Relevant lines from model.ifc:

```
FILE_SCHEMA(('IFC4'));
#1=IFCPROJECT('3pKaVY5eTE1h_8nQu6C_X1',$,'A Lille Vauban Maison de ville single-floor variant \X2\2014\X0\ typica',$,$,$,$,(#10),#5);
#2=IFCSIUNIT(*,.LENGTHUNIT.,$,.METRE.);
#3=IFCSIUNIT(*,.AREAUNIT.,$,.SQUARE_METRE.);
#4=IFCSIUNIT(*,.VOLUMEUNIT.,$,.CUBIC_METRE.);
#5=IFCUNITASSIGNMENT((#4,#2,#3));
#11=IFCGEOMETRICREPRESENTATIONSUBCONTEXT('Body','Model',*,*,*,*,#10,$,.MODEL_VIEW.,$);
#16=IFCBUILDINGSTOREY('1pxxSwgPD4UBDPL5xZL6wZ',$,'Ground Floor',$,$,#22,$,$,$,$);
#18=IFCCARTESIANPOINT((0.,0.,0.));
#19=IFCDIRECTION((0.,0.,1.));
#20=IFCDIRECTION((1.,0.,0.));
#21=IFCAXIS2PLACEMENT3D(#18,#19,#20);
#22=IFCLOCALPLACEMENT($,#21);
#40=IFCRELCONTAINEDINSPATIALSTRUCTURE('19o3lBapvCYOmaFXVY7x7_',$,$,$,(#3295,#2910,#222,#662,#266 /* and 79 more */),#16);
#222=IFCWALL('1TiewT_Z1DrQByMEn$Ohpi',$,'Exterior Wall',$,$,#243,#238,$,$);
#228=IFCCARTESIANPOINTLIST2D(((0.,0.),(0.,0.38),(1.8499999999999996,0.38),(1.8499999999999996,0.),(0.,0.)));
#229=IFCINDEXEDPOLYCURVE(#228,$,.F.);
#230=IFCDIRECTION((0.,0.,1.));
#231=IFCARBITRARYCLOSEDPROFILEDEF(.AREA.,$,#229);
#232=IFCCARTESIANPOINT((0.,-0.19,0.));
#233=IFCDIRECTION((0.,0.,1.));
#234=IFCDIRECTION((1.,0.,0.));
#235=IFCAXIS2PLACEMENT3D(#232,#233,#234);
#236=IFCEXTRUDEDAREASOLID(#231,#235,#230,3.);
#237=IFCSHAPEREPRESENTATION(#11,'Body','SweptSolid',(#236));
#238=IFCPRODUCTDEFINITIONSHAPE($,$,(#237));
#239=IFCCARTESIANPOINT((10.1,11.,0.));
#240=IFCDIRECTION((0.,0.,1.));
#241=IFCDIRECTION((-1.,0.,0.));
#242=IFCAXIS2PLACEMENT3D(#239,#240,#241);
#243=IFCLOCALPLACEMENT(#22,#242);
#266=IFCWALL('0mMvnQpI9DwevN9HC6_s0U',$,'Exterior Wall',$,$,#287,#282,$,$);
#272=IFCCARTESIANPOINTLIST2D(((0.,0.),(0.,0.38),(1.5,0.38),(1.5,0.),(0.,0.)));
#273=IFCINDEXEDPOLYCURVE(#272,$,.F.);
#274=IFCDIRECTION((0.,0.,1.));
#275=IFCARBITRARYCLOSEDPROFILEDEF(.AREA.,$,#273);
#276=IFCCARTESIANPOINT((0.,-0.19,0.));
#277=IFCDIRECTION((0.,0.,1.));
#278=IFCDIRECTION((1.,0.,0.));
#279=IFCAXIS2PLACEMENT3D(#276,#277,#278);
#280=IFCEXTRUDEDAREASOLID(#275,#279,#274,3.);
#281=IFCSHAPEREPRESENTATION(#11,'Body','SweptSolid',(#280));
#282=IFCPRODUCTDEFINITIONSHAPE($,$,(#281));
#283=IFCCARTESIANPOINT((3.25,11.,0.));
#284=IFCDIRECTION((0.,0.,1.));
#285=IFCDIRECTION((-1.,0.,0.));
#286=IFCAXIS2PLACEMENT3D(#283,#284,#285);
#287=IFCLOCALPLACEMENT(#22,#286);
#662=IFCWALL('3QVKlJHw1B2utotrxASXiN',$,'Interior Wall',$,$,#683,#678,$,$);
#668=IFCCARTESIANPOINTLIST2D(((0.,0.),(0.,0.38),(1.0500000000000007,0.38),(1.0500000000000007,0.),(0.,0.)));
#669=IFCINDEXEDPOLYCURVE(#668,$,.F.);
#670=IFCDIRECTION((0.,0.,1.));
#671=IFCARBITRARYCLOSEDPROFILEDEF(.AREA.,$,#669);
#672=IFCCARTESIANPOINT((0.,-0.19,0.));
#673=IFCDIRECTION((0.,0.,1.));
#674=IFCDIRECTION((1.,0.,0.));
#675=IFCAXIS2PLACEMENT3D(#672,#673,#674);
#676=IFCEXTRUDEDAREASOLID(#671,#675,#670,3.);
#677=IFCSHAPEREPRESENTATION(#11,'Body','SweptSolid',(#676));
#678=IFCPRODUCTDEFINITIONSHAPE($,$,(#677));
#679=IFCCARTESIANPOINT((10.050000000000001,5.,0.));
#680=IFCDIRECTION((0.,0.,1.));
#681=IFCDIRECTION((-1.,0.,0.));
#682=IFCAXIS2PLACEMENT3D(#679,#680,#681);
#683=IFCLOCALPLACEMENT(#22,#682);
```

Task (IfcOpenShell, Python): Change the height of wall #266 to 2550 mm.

```python
import ifcopenshell
import ifcopenshell.geom
import ifcopenshell.util.representation
import ifcopenshell.util.shape
import ifcopenshell.util.unit

model = ifcopenshell.open("model.ifc")
unit_scale = ifcopenshell.util.unit.calculate_unit_scale(model)
settings = ifcopenshell.geom.settings()


def volume(element):
    """Net volume in cubic metres, openings subtracted."""
    shape = ifcopenshell.geom.create_shape(settings, element)
    return ifcopenshell.util.shape.get_volume(shape.geometry)


wall = model.by_id(266)
before = volume(wall)

body = ifcopenshell.util.representation.get_representation(wall, "Model", "Body")
solid = body.Items[0]
old_height = solid.Depth
solid.Depth = 2.55 / unit_scale
after = volume(wall)

print(f"height {old_height:g} -> {solid.Depth:g}, volume {before:.3f} -> {after:.3f} m3")

model.write("model_edited.ifc")
```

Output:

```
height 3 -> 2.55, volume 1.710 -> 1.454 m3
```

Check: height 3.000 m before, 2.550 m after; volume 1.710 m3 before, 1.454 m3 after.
